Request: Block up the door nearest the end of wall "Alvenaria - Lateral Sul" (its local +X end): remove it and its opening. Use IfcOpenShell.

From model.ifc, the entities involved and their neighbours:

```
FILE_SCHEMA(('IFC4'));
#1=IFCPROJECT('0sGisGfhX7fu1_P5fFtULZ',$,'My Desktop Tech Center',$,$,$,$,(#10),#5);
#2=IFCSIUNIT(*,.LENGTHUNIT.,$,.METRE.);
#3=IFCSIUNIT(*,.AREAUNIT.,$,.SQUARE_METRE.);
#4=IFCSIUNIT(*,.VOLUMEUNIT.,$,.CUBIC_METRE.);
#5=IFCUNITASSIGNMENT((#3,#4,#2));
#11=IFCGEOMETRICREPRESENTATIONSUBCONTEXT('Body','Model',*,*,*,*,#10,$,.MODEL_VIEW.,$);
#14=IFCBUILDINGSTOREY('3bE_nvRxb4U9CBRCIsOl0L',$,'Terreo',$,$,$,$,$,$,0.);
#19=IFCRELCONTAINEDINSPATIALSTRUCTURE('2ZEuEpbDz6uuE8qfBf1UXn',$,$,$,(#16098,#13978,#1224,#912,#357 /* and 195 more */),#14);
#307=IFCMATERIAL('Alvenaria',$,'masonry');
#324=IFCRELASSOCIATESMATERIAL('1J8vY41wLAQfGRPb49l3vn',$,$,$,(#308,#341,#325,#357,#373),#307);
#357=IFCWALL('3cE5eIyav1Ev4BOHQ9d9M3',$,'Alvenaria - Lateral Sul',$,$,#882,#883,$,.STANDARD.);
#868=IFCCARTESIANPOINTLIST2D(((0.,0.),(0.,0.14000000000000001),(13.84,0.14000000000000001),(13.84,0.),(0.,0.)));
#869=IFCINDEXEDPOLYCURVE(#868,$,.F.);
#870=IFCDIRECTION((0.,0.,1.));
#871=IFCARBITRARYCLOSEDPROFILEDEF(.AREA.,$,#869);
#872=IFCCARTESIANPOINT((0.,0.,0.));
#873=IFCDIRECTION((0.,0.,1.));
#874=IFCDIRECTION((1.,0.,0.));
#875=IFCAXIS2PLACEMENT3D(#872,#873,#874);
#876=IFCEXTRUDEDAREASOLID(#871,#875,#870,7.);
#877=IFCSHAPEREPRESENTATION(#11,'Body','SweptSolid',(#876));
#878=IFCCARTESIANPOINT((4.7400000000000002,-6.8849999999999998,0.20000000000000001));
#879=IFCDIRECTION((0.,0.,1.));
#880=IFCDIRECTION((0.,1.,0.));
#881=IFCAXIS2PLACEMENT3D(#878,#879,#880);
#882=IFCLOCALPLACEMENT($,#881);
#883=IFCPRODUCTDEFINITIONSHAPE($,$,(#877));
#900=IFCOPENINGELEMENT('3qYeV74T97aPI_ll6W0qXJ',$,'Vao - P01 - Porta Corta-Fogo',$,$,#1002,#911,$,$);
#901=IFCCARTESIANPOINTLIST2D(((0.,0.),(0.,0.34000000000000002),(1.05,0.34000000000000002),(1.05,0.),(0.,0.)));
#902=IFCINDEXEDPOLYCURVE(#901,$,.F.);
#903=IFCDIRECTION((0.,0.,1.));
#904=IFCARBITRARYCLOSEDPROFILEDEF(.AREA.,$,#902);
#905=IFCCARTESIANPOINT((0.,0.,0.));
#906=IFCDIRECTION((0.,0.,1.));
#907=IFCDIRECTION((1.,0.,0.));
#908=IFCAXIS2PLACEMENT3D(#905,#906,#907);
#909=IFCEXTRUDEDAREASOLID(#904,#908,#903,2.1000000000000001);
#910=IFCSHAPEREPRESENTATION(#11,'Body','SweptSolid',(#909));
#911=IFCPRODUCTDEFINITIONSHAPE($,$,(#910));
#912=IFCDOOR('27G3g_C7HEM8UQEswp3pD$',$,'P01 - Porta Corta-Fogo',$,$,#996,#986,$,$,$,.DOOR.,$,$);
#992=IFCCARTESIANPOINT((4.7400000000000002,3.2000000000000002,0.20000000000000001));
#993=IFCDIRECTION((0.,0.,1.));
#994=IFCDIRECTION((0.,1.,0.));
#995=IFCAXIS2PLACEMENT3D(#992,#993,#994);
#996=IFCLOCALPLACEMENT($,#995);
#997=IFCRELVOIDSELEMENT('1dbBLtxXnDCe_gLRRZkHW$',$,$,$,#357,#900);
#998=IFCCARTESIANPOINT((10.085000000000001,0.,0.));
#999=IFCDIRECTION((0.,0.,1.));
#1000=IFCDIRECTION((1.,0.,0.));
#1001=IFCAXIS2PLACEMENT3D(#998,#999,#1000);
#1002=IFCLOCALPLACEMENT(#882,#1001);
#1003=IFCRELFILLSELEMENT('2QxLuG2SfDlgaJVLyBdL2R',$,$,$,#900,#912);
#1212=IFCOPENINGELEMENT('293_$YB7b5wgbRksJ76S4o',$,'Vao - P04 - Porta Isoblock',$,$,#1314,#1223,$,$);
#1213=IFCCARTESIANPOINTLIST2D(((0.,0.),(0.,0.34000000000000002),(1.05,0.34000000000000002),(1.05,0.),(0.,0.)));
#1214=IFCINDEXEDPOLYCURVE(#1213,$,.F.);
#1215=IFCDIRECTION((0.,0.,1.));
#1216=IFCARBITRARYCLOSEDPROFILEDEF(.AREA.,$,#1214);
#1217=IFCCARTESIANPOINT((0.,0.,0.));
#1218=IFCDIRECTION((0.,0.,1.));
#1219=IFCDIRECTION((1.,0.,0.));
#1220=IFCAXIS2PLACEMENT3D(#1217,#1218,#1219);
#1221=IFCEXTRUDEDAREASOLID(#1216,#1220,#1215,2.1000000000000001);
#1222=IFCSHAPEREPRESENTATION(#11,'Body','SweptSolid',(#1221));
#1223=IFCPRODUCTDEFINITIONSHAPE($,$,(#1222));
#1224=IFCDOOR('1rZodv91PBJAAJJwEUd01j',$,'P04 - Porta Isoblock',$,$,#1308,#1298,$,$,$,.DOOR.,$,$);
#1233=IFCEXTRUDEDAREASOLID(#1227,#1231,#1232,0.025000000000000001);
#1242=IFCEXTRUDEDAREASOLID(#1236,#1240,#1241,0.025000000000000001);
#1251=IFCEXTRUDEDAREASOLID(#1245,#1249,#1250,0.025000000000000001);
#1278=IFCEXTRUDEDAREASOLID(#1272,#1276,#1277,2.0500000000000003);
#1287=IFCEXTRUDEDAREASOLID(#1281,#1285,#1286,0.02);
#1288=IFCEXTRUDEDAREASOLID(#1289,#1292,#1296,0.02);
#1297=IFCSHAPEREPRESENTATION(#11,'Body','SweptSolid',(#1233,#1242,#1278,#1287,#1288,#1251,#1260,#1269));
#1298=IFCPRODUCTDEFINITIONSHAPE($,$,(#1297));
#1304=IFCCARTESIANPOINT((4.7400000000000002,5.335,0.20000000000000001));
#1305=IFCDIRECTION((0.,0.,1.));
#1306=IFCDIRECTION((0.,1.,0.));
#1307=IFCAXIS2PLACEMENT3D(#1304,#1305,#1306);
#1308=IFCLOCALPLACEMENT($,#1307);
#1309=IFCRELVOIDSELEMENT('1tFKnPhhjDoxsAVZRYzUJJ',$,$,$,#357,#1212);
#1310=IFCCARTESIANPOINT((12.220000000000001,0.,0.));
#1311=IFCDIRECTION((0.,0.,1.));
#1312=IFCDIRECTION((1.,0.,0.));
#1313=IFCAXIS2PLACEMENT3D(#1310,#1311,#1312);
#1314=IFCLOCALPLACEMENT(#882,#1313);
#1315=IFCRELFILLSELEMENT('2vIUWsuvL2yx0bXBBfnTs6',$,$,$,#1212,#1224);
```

```python
import ifcopenshell
import ifcopenshell.api.feature
import ifcopenshell.api.root
import ifcopenshell.geom
import ifcopenshell.util.shape

model = ifcopenshell.open("model.ifc")
settings = ifcopenshell.geom.settings()


def volume(element):
    """Net volume in cubic metres, openings subtracted."""
    shape = ifcopenshell.geom.create_shape(settings, element)
    return ifcopenshell.util.shape.get_volume(shape.geometry)


door = model.by_guid("1rZodv91PBJAAJJwEUd01j")
opening = door.FillsVoids[0].RelatingOpeningElement
wall = opening.VoidsElements[0].RelatingBuildingElement
before = volume(wall)

ifcopenshell.api.root.remove_product(model, product=door)
ifcopenshell.api.feature.remove_feature(model, feature=opening)

after = volume(wall)

print(f"wall volume {before:.3f} -> {after:.3f} m3")

model.write("model-out.ifc")
```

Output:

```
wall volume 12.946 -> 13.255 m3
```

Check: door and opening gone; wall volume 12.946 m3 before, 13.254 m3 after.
